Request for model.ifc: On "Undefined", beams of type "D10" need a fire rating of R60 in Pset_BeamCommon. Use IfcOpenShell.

First a look at what the model holds.

```python
import ifcopenshell
import ifcopenshell.util.element

model = ifcopenshell.open("model.ifc")
print(model.schema)
storey = next(s for s in model.by_type("IfcBuildingStorey") if s.Name == "Undefined")
beams = [e for e in ifcopenshell.util.element.get_decomposition(storey) if e.is_a("IfcBeam")]
seen = {}
for e in beams:
    element_type = ifcopenshell.util.element.get_type(e)
    key = (element_type.Name if element_type != e and element_type else None, ifcopenshell.util.element.get_pset(e, "Pset_BeamCommon", "FireRating"))
    seen[key] = seen.get(key, 0) + 1
for (name, value), count in sorted(seen.items(), key=str):
    print(count, "x", name, "|", value)
```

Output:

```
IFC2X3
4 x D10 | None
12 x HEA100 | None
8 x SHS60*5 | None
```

```python
import ifcopenshell
import ifcopenshell.api.pset
import ifcopenshell.util.element

model = ifcopenshell.open("model.ifc")

storey = next(s for s in model.by_type("IfcBuildingStorey") if s.Name == "Undefined")
beams = [e for e in ifcopenshell.util.element.get_decomposition(storey) if e.is_a("IfcBeam")]

count = 0
for e in beams:
    element_type = ifcopenshell.util.element.get_type(e)
    if element_type in (None, e) or element_type.Name != "D10":
        continue
    # add_pset returns the element's existing set when there is one.
    pset = ifcopenshell.api.pset.add_pset(model, product=e, name="Pset_BeamCommon")
    ifcopenshell.api.pset.edit_pset(model, pset=pset, properties={"FireRating": "R60"})
    count += 1

print(count, "beams updated")

model.write("model-out.ifc")
```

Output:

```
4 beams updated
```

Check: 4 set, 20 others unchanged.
